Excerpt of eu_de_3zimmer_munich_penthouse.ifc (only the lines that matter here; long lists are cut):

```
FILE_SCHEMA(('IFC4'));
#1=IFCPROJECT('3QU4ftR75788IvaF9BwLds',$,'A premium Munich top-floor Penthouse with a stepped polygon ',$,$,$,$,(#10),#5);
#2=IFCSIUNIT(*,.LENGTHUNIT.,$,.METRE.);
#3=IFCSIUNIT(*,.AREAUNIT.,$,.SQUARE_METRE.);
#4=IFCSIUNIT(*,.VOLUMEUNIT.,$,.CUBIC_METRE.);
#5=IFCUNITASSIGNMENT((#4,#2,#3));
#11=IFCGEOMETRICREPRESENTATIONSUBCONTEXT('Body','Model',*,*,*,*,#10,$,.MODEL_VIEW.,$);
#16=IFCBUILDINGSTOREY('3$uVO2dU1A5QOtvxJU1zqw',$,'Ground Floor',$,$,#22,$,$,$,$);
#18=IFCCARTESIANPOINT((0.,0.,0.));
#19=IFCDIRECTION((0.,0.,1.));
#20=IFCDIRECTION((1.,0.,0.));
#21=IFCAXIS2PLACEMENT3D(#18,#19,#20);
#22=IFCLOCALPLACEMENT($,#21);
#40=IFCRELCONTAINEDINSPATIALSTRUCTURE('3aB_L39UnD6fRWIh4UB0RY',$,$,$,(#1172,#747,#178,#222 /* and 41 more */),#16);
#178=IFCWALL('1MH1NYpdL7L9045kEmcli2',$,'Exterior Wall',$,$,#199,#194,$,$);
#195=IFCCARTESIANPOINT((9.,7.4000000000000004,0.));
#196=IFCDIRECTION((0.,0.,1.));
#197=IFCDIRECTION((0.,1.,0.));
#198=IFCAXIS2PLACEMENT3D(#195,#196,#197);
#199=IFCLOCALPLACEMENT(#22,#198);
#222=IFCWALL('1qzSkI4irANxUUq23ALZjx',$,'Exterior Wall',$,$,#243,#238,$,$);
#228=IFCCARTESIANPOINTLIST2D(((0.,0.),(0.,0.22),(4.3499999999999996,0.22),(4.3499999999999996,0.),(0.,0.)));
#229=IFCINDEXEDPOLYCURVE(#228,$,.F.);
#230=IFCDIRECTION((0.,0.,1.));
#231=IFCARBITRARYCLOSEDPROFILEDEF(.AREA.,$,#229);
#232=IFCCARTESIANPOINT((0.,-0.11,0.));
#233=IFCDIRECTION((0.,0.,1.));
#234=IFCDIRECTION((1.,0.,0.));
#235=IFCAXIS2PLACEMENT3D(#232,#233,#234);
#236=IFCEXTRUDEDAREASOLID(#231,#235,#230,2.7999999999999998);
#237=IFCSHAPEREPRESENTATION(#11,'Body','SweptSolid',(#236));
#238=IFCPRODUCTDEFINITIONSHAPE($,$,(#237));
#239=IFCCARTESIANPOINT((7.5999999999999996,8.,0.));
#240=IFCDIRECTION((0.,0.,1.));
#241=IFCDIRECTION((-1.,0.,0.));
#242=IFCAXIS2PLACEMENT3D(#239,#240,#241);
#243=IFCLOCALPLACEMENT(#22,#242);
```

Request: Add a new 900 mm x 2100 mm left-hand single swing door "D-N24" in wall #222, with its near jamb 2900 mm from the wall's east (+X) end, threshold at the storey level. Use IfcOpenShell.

```python
import numpy as np
import ifcopenshell
import ifcopenshell.api.feature
import ifcopenshell.api.geometry
import ifcopenshell.api.root
import ifcopenshell.api.spatial
import ifcopenshell.geom
import ifcopenshell.util.element
import ifcopenshell.util.placement
import ifcopenshell.util.representation
import ifcopenshell.util.shape
import ifcopenshell.util.unit

model = ifcopenshell.open("eu_de_3zimmer_munich_penthouse.ifc")
unit_scale = ifcopenshell.util.unit.calculate_unit_scale(model)
settings = ifcopenshell.geom.settings()


def volume(element):
    """Net volume in cubic metres, openings subtracted."""
    shape = ifcopenshell.geom.create_shape(settings, element)
    return ifcopenshell.util.shape.get_volume(shape.geometry)


wall = model.by_guid("1qzSkI4irANxUUq23ALZjx")
storey = ifcopenshell.util.element.get_container(wall, ifc_class="IfcBuildingStorey")
context = ifcopenshell.util.representation.get_context(model, "Model", "Body", "MODEL_VIEW")
before = volume(wall)

width, height, from_end, sill = 0.9, 2.1, 2.9, 0.0  # metres

# The wall runs along its own X axis, and the end named is its -X end.
wall_shape = ifcopenshell.geom.create_shape(settings, wall)
x, y, z = ifcopenshell.util.shape.get_vertices(wall_shape.geometry).T
start = x.min() + from_end
face, thickness = float(y.min()), float(y.max() - y.min())
wall_matrix = ifcopenshell.util.placement.get_local_placement(wall.ObjectPlacement)
level = ifcopenshell.util.placement.get_local_placement(storey.ObjectPlacement)[2, 3]


def in_wall(x, y):
    """Placement at x, y metres in the wall's axes, at sill height."""
    matrix = wall_matrix.copy()
    matrix[:, 3] = wall_matrix @ np.array([x / unit_scale, y / unit_scale, 0.0, 1.0])
    matrix[2, 3] = level + sill / unit_scale
    return matrix


# Opening: a box that overshoots both wall faces by 50 mm.
opening = ifcopenshell.api.root.create_entity(model, ifc_class="IfcOpeningElement", predefined_type="OPENING")
box = ifcopenshell.api.geometry.add_wall_representation(
    model, context=context, length=width, height=height, thickness=thickness + 0.1
)
ifcopenshell.api.geometry.assign_representation(model, product=opening, representation=box)
ifcopenshell.api.geometry.edit_object_placement(model, product=opening, matrix=in_wall(start, face - 0.05), is_si=False)
ifcopenshell.api.feature.add_feature(model, feature=opening, element=wall)

door = ifcopenshell.api.root.create_entity(model, ifc_class="IfcDoor", name="D-N24", predefined_type="DOOR")
door.OverallWidth, door.OverallHeight = width / unit_scale, height / unit_scale
door.OperationType = "SINGLE_SWING_LEFT"
body = ifcopenshell.api.geometry.add_door_representation(
    model,
    context=context,
    overall_width=door.OverallWidth,
    overall_height=door.OverallHeight,
    operation_type="SINGLE_SWING_LEFT",
    lining_properties={"LiningDepth": thickness / unit_scale, "ThresholdDepth": thickness / unit_scale},
)
ifcopenshell.api.geometry.assign_representation(model, product=door, representation=body)
ifcopenshell.api.spatial.assign_container(model, products=[door], relating_structure=storey)
ifcopenshell.api.feature.add_filling(model, opening=opening, element=door)

# The lining spans the wall, so the door starts at the wall face.
ifcopenshell.api.geometry.edit_object_placement(model, product=door, matrix=in_wall(start, face), is_si=False)

after = volume(wall)

print(f"wall volume {before:.3f} -> {after:.3f} m3")

model.write("eu_de_3zimmer_munich_penthouse_v2.ifc")
```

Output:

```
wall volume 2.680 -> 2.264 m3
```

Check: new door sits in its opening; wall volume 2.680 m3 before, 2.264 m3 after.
